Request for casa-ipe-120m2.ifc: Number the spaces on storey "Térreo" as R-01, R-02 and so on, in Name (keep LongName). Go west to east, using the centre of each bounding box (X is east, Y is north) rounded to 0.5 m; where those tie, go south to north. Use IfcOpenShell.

First a look at what the model holds.

```python
import ifcopenshell
import ifcopenshell.util.element
import ifcopenshell.util.placement

model = ifcopenshell.open("casa-ipe-120m2.ifc")
print(model.schema)
storey = next(s for s in model.by_type("IfcBuildingStorey") if s.Name == "Térreo")
spaces = [e for e in ifcopenshell.util.element.get_decomposition(storey) if e.is_a("IfcSpace")]
for e in sorted(spaces, key=lambda e: e.id()):
    origin = ifcopenshell.util.placement.get_local_placement(e.ObjectPlacement)[:3, 3]
    print(e.id(), e.Name, e.LongName, origin.round(2) + 0.0, sep=" | ")
```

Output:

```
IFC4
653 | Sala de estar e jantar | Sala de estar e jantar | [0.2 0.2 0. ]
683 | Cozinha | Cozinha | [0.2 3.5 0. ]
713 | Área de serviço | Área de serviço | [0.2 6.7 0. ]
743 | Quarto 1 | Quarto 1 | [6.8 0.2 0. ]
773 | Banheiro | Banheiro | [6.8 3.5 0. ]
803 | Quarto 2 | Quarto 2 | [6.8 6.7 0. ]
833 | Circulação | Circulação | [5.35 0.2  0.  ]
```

```python
import ifcopenshell
import ifcopenshell.geom
import ifcopenshell.util.element
import ifcopenshell.util.shape

model = ifcopenshell.open("casa-ipe-120m2.ifc")
settings = ifcopenshell.geom.settings()
settings.set("use-world-coords", True)


def centre(element):
    shape = ifcopenshell.geom.create_shape(settings, element)
    return ifcopenshell.util.shape.get_bbox_centroid(shape.geometry)


storey = next(s for s in model.by_type("IfcBuildingStorey") if s.Name == "Térreo")
spaces = [e for e in ifcopenshell.util.element.get_decomposition(storey) if e.is_a("IfcSpace")]

# Insertion points can sit at a corner or the storey origin, so sort by the geometry (in metres).
centres = {e: centre(e) for e in spaces}
spaces.sort(key=lambda e: (round(centres[e][0] / 0.5), centres[e][1]))

for i, e in enumerate(spaces, start=1):
    number = f"R-{i:02d}"
    e.Name = number
    print(e.id(), number)

model.write("casa-ipe-120m2_rev.ifc")
```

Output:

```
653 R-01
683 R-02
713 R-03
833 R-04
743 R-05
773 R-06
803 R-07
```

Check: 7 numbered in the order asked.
